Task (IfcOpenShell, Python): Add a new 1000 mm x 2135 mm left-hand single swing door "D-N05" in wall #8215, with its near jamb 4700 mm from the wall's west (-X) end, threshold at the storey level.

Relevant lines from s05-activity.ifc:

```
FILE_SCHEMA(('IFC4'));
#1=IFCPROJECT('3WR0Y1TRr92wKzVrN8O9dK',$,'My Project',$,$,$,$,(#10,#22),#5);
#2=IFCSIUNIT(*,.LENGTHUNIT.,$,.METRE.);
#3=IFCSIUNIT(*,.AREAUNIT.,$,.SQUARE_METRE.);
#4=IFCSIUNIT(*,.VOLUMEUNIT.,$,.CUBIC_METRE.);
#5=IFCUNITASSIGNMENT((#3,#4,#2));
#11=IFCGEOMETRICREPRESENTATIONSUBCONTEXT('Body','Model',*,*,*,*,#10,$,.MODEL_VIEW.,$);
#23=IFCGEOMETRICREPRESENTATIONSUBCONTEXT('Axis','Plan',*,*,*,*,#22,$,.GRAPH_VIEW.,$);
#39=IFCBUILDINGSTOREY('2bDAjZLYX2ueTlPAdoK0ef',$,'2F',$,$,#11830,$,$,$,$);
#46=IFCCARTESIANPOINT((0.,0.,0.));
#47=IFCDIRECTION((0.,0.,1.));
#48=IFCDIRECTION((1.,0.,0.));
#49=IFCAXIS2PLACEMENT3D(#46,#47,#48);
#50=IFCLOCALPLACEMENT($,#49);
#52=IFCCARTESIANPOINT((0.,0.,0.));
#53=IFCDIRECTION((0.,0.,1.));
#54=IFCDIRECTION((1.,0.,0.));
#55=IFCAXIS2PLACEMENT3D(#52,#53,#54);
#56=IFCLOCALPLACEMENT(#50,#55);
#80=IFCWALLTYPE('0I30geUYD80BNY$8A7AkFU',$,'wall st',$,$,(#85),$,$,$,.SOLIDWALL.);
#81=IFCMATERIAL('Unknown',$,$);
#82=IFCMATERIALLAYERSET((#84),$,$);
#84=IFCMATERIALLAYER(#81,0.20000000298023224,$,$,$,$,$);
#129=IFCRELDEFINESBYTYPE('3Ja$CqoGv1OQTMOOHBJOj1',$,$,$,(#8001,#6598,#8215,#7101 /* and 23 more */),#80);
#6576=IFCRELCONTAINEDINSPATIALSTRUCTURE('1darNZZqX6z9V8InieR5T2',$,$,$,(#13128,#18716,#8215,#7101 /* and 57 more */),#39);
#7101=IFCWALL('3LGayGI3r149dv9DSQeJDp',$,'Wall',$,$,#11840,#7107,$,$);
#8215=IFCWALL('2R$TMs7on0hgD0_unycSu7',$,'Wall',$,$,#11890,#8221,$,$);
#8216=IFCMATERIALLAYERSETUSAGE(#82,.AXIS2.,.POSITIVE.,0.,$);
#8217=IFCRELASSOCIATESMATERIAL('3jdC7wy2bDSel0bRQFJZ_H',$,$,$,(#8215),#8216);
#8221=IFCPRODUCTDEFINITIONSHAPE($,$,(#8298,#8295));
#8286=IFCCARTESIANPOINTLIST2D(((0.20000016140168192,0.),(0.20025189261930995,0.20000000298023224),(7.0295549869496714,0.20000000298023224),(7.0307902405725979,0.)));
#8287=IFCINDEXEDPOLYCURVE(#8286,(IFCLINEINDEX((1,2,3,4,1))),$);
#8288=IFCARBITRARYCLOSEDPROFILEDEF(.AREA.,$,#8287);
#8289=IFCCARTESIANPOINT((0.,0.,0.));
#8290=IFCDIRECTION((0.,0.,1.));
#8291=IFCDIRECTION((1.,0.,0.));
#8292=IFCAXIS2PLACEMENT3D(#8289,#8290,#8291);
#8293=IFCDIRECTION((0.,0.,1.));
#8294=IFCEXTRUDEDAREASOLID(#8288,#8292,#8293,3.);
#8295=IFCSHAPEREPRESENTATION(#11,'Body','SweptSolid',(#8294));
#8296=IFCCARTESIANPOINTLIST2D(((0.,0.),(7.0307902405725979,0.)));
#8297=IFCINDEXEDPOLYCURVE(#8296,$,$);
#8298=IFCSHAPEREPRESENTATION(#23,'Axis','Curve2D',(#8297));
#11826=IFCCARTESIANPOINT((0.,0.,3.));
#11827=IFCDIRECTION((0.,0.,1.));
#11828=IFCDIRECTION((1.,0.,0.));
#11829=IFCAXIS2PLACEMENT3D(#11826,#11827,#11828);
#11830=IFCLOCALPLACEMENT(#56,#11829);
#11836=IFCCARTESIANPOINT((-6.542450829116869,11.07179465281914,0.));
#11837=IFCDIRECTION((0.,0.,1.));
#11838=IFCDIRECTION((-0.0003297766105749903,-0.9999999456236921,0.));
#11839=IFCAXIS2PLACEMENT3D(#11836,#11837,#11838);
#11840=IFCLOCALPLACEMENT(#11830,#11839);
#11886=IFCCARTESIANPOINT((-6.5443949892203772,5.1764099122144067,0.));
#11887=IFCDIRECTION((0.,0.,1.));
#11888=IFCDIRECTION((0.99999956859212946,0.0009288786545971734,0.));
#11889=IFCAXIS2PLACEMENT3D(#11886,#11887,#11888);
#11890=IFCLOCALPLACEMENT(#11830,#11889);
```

```python
import numpy as np
import ifcopenshell
import ifcopenshell.api.feature
import ifcopenshell.api.geometry
import ifcopenshell.api.root
import ifcopenshell.api.spatial
import ifcopenshell.geom
import ifcopenshell.util.element
import ifcopenshell.util.placement
import ifcopenshell.util.representation
import ifcopenshell.util.shape
import ifcopenshell.util.unit

model = ifcopenshell.open("s05-activity.ifc")
unit_scale = ifcopenshell.util.unit.calculate_unit_scale(model)
settings = ifcopenshell.geom.settings()


def volume(element):
    """Net volume in cubic metres, openings subtracted."""
    shape = ifcopenshell.geom.create_shape(settings, element)
    return ifcopenshell.util.shape.get_volume(shape.geometry)


wall = model.by_id(8215)
storey = ifcopenshell.util.element.get_container(wall, ifc_class="IfcBuildingStorey")
context = ifcopenshell.util.representation.get_context(model, "Model", "Body", "MODEL_VIEW")
before = volume(wall)

width, height, from_end, sill = 1, 2.135, 4.7, 0.0  # metres

# The wall runs along its own X axis, and the end named is its -X end.
wall_shape = ifcopenshell.geom.create_shape(settings, wall)
x, y, z = ifcopenshell.util.shape.get_vertices(wall_shape.geometry).T
start = x.min() + from_end
face, thickness = float(y.min()), float(y.max() - y.min())
wall_matrix = ifcopenshell.util.placement.get_local_placement(wall.ObjectPlacement)
level = ifcopenshell.util.placement.get_local_placement(storey.ObjectPlacement)[2, 3]


def in_wall(x, y):
    """Placement at x, y metres in the wall's axes, at sill height."""
    matrix = wall_matrix.copy()
    matrix[:, 3] = wall_matrix @ np.array([x / unit_scale, y / unit_scale, 0.0, 1.0])
    matrix[2, 3] = level + sill / unit_scale
    return matrix


# Opening: a box that overshoots both wall faces by 50 mm.
opening = ifcopenshell.api.root.create_entity(model, ifc_class="IfcOpeningElement", predefined_type="OPENING")
box = ifcopenshell.api.geometry.add_wall_representation(
    model, context=context, length=width, height=height, thickness=thickness + 0.1
)
ifcopenshell.api.geometry.assign_representation(model, product=opening, representation=box)
ifcopenshell.api.geometry.edit_object_placement(model, product=opening, matrix=in_wall(start, face - 0.05), is_si=False)
ifcopenshell.api.feature.add_feature(model, feature=opening, element=wall)

door = ifcopenshell.api.root.create_entity(model, ifc_class="IfcDoor", name="D-N05", predefined_type="DOOR")
door.OverallWidth, door.OverallHeight = width / unit_scale, height / unit_scale
door.OperationType = "SINGLE_SWING_LEFT"
body = ifcopenshell.api.geometry.add_door_representation(
    model,
    context=context,
    overall_width=door.OverallWidth,
    overall_height=door.OverallHeight,
    operation_type="SINGLE_SWING_LEFT",
    lining_properties={"LiningDepth": thickness / unit_scale, "ThresholdDepth": thickness / unit_scale},
)
ifcopenshell.api.geometry.assign_representation(model, product=door, representation=body)
ifcopenshell.api.spatial.assign_container(model, products=[door], relating_structure=storey)
ifcopenshell.api.feature.add_filling(model, opening=opening, element=door)

# The lining spans the wall, so the door starts at the wall face.
ifcopenshell.api.geometry.edit_object_placement(model, product=door, matrix=in_wall(start, face), is_si=False)

after = volume(wall)

print(f"wall volume {before:.3f} -> {after:.3f} m3")

model.write("s05-activity-out.ifc")
```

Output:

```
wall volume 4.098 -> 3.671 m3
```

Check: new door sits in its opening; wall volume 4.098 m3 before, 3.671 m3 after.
